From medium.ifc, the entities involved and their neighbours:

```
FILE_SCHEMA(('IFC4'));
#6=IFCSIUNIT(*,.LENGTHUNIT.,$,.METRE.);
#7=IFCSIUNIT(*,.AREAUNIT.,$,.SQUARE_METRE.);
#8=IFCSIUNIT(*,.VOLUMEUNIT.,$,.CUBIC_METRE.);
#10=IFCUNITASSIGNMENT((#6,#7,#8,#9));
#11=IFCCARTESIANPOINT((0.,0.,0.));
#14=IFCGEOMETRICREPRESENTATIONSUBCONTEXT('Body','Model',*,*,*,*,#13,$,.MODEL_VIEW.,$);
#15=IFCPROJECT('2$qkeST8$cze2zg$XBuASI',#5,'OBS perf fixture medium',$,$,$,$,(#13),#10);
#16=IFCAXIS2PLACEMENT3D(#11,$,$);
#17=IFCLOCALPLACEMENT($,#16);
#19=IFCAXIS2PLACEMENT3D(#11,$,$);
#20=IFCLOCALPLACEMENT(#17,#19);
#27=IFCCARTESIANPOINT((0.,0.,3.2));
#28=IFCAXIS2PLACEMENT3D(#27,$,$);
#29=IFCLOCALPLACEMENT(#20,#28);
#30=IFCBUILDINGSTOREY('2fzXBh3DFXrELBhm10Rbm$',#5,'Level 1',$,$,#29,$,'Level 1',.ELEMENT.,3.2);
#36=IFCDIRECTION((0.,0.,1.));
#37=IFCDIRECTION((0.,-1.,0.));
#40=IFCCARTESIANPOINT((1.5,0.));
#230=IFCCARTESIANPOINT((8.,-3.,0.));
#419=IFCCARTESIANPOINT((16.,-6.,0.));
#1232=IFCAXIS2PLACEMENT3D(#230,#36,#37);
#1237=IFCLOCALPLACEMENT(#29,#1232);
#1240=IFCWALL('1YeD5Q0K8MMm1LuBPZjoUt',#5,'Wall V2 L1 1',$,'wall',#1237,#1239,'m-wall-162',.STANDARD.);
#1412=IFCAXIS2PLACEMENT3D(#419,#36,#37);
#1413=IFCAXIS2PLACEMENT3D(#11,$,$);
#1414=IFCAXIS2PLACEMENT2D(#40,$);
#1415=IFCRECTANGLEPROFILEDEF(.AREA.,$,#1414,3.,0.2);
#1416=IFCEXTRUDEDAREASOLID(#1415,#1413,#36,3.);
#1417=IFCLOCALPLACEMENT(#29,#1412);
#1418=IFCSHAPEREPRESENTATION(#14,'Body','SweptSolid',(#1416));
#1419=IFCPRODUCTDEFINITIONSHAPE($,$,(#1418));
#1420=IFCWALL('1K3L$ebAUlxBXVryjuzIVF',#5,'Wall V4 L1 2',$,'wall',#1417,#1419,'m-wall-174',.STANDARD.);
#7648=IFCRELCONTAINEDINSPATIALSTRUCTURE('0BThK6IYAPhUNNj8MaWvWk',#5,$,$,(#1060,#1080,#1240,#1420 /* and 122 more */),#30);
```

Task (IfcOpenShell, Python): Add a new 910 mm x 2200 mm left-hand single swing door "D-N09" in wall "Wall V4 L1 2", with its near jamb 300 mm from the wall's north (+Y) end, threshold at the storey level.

```python
import numpy as np
import ifcopenshell
import ifcopenshell.api.feature
import ifcopenshell.api.geometry
import ifcopenshell.api.root
import ifcopenshell.api.spatial
import ifcopenshell.geom
import ifcopenshell.util.element
import ifcopenshell.util.placement
import ifcopenshell.util.representation
import ifcopenshell.util.shape
import ifcopenshell.util.unit

model = ifcopenshell.open("medium.ifc")
unit_scale = ifcopenshell.util.unit.calculate_unit_scale(model)
settings = ifcopenshell.geom.settings()


def volume(element):
    """Net volume in cubic metres, openings subtracted."""
    shape = ifcopenshell.geom.create_shape(settings, element)
    return ifcopenshell.util.shape.get_volume(shape.geometry)


wall = model.by_guid("1K3L$ebAUlxBXVryjuzIVF")
storey = ifcopenshell.util.element.get_container(wall, ifc_class="IfcBuildingStorey")
context = ifcopenshell.util.representation.get_context(model, "Model", "Body", "MODEL_VIEW")
before = volume(wall)

width, height, from_end, sill = 0.91, 2.2, 0.3, 0.0  # metres

# The wall runs along its own X axis, and the end named is its -X end.
wall_shape = ifcopenshell.geom.create_shape(settings, wall)
x, y, z = ifcopenshell.util.shape.get_vertices(wall_shape.geometry).T
start = x.min() + from_end
face, thickness = float(y.min()), float(y.max() - y.min())
wall_matrix = ifcopenshell.util.placement.get_local_placement(wall.ObjectPlacement)
level = ifcopenshell.util.placement.get_local_placement(storey.ObjectPlacement)[2, 3]


def in_wall(x, y):
    """Placement at x, y metres in the wall's axes, at sill height."""
    matrix = wall_matrix.copy()
    matrix[:, 3] = wall_matrix @ np.array([x / unit_scale, y / unit_scale, 0.0, 1.0])
    matrix[2, 3] = level + sill / unit_scale
    return matrix


# Opening: a box that overshoots both wall faces by 50 mm.
opening = ifcopenshell.api.root.create_entity(model, ifc_class="IfcOpeningElement", predefined_type="OPENING")
box = ifcopenshell.api.geometry.add_wall_representation(
    model, context=context, length=width, height=height, thickness=thickness + 0.1
)
ifcopenshell.api.geometry.assign_representation(model, product=opening, representation=box)
ifcopenshell.api.geometry.edit_object_placement(model, product=opening, matrix=in_wall(start, face - 0.05), is_si=False)
ifcopenshell.api.feature.add_feature(model, feature=opening, element=wall)

door = ifcopenshell.api.root.create_entity(model, ifc_class="IfcDoor", name="D-N09", predefined_type="DOOR")
door.OverallWidth, door.OverallHeight = width / unit_scale, height / unit_scale
door.OperationType = "SINGLE_SWING_LEFT"
body = ifcopenshell.api.geometry.add_door_representation(
    model,
    context=context,
    overall_width=door.OverallWidth,
    overall_height=door.OverallHeight,
    operation_type="SINGLE_SWING_LEFT",
    lining_properties={"LiningDepth": thickness / unit_scale, "ThresholdDepth": thickness / unit_scale},
)
ifcopenshell.api.geometry.assign_representation(model, product=door, representation=body)
ifcopenshell.api.spatial.assign_container(model, products=[door], relating_structure=storey)
ifcopenshell.api.feature.add_filling(model, opening=opening, element=door)

# The lining spans the wall, so the door starts at the wall face.
ifcopenshell.api.geometry.edit_object_placement(model, product=door, matrix=in_wall(start, face), is_si=False)

after = volume(wall)

print(f"wall volume {before:.3f} -> {after:.3f} m3")

model.write("medium_rev.ifc")
```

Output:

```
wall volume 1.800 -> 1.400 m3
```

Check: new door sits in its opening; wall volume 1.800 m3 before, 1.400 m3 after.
